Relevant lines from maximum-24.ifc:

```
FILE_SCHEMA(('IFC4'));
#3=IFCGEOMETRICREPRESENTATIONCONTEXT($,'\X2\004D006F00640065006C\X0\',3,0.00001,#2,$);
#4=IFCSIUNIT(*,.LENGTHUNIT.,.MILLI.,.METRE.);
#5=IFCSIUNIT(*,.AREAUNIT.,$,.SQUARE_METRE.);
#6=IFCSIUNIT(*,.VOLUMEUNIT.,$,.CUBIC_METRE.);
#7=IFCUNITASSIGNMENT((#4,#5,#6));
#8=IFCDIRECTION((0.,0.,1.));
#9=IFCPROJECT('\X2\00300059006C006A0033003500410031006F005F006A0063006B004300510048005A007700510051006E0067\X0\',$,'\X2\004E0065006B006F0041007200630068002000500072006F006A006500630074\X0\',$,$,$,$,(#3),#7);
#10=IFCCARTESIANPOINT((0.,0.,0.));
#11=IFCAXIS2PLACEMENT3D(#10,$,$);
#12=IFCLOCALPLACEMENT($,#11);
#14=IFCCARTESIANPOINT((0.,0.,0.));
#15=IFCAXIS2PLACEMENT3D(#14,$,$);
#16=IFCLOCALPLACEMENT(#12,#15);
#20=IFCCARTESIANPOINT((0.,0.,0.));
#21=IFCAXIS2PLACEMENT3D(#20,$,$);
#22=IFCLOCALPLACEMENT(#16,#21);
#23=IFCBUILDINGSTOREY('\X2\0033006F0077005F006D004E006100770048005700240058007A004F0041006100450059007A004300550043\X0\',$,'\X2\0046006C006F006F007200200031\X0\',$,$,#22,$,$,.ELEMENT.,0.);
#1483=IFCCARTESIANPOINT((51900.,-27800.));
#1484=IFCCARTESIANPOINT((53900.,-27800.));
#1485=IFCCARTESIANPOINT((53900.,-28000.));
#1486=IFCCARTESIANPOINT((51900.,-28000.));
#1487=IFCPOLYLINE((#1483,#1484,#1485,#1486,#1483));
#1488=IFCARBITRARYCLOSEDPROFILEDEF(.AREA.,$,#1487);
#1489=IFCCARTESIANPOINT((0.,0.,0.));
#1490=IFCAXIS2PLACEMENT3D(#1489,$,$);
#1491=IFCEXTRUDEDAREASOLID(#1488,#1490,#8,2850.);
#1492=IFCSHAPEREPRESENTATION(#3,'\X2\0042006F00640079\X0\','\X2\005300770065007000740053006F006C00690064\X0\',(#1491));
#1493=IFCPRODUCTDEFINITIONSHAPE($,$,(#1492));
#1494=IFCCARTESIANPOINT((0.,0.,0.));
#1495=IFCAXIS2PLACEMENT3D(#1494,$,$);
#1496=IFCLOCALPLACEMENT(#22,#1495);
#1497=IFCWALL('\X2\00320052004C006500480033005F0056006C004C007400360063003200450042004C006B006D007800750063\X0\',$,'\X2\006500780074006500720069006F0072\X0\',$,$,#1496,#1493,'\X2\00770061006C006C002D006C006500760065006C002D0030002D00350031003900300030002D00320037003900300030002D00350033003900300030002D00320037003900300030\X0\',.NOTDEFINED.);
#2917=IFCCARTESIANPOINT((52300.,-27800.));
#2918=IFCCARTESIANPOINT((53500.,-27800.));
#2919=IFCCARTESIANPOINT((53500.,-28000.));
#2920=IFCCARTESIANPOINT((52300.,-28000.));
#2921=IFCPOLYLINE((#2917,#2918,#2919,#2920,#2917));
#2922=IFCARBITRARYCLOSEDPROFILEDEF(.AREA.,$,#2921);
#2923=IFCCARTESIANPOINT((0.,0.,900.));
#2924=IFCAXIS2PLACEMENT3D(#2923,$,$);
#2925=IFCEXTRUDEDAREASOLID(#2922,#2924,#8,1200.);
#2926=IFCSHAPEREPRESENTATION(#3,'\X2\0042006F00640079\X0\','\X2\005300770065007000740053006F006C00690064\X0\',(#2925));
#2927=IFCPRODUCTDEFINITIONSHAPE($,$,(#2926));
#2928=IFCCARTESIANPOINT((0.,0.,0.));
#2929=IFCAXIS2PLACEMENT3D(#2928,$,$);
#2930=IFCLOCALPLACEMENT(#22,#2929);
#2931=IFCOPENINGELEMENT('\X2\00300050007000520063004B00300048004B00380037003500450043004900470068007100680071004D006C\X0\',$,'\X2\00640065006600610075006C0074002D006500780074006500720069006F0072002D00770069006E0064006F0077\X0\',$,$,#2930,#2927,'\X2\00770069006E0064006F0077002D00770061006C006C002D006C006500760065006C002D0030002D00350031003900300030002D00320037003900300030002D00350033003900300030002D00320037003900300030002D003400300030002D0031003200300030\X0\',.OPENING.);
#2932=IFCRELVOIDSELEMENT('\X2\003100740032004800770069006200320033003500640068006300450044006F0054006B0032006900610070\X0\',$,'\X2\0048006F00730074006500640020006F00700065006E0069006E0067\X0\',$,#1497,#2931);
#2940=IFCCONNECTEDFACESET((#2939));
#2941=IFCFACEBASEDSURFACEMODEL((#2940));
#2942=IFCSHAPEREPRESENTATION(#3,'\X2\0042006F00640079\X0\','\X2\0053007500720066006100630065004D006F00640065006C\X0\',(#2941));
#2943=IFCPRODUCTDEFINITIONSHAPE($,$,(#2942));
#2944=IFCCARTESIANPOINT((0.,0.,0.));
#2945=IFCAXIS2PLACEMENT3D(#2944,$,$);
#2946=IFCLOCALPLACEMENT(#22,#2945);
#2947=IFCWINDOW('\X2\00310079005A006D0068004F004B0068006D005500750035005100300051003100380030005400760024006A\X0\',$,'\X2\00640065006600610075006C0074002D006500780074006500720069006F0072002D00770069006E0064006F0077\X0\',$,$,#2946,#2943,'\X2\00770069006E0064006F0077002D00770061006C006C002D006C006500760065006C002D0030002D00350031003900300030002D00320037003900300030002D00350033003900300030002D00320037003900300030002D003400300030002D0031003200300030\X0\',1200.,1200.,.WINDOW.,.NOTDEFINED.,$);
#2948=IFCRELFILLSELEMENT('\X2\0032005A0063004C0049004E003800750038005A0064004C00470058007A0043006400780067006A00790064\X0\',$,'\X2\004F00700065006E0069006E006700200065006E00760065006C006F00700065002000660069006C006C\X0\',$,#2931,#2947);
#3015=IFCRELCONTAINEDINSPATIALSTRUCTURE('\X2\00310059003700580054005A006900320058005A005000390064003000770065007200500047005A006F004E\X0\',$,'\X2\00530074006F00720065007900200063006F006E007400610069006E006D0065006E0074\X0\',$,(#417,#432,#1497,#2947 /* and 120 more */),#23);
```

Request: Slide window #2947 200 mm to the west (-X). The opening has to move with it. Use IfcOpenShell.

```python
import ifcopenshell
import ifcopenshell.api.geometry
import ifcopenshell.util.placement
import ifcopenshell.util.unit

model = ifcopenshell.open("maximum-24.ifc")
unit_scale = ifcopenshell.util.unit.calculate_unit_scale(model)

window = model.by_guid("1yZmhOKhmUu5Q0Q180Tv$j")
opening = window.FillsVoids[0].RelatingOpeningElement
wall = opening.VoidsElements[0].RelatingBuildingElement

wall_matrix = ifcopenshell.util.placement.get_local_placement(wall.ObjectPlacement)
shift = wall_matrix[:3, 0] * -0.2 / unit_scale
before = ifcopenshell.util.placement.get_local_placement(window.ObjectPlacement)[:3, 3].copy()

# The window is not placed relative to its opening, so move both.
for product in (opening, window):
    matrix = ifcopenshell.util.placement.get_local_placement(product.ObjectPlacement)
    matrix[:3, 3] += shift
    ifcopenshell.api.geometry.edit_object_placement(model, product=product, matrix=matrix, is_si=False)

after = ifcopenshell.util.placement.get_local_placement(window.ObjectPlacement)[:3, 3]
print("window moved by", (after - before).round(3) + 0.0)

model.write("maximum-24_updated.ifc")
```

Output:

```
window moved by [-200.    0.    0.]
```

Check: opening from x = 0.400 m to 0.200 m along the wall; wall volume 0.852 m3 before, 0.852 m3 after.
